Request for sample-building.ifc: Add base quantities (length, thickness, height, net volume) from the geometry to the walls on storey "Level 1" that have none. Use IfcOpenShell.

First a look at what the model holds.

```python
import ifcopenshell
import ifcopenshell.util.element
import ifcopenshell.util.unit

model = ifcopenshell.open("sample-building.ifc")
print(model.schema)
for unit_type in ("LENGTHUNIT", "AREAUNIT", "VOLUMEUNIT"):
    print(unit_type, ifcopenshell.util.unit.calculate_unit_scale(model, unit_type))
storey = next(s for s in model.by_type("IfcBuildingStorey") if s.Name == "Level 1")
walls = [e for e in ifcopenshell.util.element.get_decomposition(storey) if e.is_a("IfcWall")]
for e in sorted(walls, key=lambda e: e.id()):
    print(e.id(), e.is_a(), e.Name, list(ifcopenshell.util.element.get_psets(e, qtos_only=True)), sep=" | ")
```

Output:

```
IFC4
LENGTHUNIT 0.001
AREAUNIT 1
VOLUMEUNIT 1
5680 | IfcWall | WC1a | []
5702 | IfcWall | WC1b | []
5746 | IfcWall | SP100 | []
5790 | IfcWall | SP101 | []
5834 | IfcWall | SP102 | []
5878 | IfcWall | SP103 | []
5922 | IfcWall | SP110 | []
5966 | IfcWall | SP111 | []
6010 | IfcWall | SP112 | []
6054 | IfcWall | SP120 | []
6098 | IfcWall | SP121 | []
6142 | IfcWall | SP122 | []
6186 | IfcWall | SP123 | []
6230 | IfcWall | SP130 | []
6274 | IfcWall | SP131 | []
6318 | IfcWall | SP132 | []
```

```python
import ifcopenshell
import ifcopenshell.api.pset
import ifcopenshell.geom
import ifcopenshell.util.element
import ifcopenshell.util.shape
import ifcopenshell.util.unit

model = ifcopenshell.open("sample-building.ifc")
unit_scale = ifcopenshell.util.unit.calculate_unit_scale(model)
volume_scale = ifcopenshell.util.unit.calculate_unit_scale(model, "VOLUMEUNIT")
settings = ifcopenshell.geom.settings()

storey = next(s for s in model.by_type("IfcBuildingStorey") if s.Name == "Level 1")
walls = [e for e in ifcopenshell.util.element.get_decomposition(storey) if e.is_a("IfcWall")]

for e in sorted(walls, key=lambda e: e.id()):
    if ifcopenshell.util.element.get_psets(e, qtos_only=True, should_inherit=False):
        continue
    # Geometry comes back in metres, in the element's own axes.
    shape = ifcopenshell.geom.create_shape(settings, e)
    values = {
        "Length": ifcopenshell.util.shape.get_x(shape.geometry) / unit_scale,
        "Width": ifcopenshell.util.shape.get_y(shape.geometry) / unit_scale,
        "Height": ifcopenshell.util.shape.get_z(shape.geometry) / unit_scale,
        "NetVolume": ifcopenshell.util.shape.get_volume(shape.geometry) / volume_scale,
    }
    qto = ifcopenshell.api.pset.add_qto(model, product=e, name="Qto_WallBaseQuantities")
    ifcopenshell.api.pset.edit_qto(model, qto=qto, properties=values)
    print(e.id(), {k: round(v, 3) for k, v in values.items()})

model.write("sample-building_v2.ifc")
```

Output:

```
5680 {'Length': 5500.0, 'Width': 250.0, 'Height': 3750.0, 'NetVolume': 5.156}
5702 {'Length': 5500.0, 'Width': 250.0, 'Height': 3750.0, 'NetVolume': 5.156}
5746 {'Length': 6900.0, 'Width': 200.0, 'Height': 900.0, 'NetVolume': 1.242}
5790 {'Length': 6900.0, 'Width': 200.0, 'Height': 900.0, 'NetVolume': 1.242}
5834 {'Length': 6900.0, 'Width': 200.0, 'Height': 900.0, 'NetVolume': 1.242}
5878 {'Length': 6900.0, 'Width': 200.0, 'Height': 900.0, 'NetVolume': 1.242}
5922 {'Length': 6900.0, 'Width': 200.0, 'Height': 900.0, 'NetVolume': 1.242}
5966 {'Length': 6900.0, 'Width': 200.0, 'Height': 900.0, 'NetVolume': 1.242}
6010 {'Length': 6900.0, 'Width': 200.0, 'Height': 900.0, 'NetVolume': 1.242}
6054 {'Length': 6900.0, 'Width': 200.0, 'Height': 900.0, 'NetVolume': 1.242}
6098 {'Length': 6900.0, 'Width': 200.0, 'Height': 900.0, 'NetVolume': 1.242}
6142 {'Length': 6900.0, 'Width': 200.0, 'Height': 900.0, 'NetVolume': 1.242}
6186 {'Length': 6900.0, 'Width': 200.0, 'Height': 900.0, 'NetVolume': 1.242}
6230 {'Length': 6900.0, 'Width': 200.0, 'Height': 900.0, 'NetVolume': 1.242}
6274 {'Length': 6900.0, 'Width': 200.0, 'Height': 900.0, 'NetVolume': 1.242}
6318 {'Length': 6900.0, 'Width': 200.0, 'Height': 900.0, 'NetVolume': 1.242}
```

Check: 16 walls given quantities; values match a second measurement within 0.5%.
